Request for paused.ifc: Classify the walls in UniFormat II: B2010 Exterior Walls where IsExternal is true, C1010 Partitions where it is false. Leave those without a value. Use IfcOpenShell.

First a look at what the model holds.

```python
import ifcopenshell
import ifcopenshell.util.element

model = ifcopenshell.open("paused.ifc")
print(model.schema)
print("classifications:", [c.Name for c in model.by_type("IfcClassification")])
values = [ifcopenshell.util.element.get_pset(e, "Pset_WallCommon", "IsExternal") for e in model.by_type("IfcWall")]
for value in (True, False, None):
    print("IsExternal", value, values.count(value))
```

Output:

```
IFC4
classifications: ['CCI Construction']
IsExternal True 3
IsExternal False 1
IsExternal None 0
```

```python
import ifcopenshell
import ifcopenshell.api.classification
import ifcopenshell.util.element

model = ifcopenshell.open("paused.ifc")

system = ifcopenshell.api.classification.add_classification(model, classification="UniFormat II")

walls = model.by_type("IfcWall")
external = {e: ifcopenshell.util.element.get_pset(e, "Pset_WallCommon", "IsExternal") for e in walls}
for flag, code, name in ((True, "B2010", "Exterior Walls"), (False, "C1010", "Partitions")):
    products = [e for e in walls if external[e] is flag]
    ifcopenshell.api.classification.add_reference(
        model, products=products, classification=system, identification=code, name=name
    )
    print(code, len(products))

model.write("paused_edited.ifc")
```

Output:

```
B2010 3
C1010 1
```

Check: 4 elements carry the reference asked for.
